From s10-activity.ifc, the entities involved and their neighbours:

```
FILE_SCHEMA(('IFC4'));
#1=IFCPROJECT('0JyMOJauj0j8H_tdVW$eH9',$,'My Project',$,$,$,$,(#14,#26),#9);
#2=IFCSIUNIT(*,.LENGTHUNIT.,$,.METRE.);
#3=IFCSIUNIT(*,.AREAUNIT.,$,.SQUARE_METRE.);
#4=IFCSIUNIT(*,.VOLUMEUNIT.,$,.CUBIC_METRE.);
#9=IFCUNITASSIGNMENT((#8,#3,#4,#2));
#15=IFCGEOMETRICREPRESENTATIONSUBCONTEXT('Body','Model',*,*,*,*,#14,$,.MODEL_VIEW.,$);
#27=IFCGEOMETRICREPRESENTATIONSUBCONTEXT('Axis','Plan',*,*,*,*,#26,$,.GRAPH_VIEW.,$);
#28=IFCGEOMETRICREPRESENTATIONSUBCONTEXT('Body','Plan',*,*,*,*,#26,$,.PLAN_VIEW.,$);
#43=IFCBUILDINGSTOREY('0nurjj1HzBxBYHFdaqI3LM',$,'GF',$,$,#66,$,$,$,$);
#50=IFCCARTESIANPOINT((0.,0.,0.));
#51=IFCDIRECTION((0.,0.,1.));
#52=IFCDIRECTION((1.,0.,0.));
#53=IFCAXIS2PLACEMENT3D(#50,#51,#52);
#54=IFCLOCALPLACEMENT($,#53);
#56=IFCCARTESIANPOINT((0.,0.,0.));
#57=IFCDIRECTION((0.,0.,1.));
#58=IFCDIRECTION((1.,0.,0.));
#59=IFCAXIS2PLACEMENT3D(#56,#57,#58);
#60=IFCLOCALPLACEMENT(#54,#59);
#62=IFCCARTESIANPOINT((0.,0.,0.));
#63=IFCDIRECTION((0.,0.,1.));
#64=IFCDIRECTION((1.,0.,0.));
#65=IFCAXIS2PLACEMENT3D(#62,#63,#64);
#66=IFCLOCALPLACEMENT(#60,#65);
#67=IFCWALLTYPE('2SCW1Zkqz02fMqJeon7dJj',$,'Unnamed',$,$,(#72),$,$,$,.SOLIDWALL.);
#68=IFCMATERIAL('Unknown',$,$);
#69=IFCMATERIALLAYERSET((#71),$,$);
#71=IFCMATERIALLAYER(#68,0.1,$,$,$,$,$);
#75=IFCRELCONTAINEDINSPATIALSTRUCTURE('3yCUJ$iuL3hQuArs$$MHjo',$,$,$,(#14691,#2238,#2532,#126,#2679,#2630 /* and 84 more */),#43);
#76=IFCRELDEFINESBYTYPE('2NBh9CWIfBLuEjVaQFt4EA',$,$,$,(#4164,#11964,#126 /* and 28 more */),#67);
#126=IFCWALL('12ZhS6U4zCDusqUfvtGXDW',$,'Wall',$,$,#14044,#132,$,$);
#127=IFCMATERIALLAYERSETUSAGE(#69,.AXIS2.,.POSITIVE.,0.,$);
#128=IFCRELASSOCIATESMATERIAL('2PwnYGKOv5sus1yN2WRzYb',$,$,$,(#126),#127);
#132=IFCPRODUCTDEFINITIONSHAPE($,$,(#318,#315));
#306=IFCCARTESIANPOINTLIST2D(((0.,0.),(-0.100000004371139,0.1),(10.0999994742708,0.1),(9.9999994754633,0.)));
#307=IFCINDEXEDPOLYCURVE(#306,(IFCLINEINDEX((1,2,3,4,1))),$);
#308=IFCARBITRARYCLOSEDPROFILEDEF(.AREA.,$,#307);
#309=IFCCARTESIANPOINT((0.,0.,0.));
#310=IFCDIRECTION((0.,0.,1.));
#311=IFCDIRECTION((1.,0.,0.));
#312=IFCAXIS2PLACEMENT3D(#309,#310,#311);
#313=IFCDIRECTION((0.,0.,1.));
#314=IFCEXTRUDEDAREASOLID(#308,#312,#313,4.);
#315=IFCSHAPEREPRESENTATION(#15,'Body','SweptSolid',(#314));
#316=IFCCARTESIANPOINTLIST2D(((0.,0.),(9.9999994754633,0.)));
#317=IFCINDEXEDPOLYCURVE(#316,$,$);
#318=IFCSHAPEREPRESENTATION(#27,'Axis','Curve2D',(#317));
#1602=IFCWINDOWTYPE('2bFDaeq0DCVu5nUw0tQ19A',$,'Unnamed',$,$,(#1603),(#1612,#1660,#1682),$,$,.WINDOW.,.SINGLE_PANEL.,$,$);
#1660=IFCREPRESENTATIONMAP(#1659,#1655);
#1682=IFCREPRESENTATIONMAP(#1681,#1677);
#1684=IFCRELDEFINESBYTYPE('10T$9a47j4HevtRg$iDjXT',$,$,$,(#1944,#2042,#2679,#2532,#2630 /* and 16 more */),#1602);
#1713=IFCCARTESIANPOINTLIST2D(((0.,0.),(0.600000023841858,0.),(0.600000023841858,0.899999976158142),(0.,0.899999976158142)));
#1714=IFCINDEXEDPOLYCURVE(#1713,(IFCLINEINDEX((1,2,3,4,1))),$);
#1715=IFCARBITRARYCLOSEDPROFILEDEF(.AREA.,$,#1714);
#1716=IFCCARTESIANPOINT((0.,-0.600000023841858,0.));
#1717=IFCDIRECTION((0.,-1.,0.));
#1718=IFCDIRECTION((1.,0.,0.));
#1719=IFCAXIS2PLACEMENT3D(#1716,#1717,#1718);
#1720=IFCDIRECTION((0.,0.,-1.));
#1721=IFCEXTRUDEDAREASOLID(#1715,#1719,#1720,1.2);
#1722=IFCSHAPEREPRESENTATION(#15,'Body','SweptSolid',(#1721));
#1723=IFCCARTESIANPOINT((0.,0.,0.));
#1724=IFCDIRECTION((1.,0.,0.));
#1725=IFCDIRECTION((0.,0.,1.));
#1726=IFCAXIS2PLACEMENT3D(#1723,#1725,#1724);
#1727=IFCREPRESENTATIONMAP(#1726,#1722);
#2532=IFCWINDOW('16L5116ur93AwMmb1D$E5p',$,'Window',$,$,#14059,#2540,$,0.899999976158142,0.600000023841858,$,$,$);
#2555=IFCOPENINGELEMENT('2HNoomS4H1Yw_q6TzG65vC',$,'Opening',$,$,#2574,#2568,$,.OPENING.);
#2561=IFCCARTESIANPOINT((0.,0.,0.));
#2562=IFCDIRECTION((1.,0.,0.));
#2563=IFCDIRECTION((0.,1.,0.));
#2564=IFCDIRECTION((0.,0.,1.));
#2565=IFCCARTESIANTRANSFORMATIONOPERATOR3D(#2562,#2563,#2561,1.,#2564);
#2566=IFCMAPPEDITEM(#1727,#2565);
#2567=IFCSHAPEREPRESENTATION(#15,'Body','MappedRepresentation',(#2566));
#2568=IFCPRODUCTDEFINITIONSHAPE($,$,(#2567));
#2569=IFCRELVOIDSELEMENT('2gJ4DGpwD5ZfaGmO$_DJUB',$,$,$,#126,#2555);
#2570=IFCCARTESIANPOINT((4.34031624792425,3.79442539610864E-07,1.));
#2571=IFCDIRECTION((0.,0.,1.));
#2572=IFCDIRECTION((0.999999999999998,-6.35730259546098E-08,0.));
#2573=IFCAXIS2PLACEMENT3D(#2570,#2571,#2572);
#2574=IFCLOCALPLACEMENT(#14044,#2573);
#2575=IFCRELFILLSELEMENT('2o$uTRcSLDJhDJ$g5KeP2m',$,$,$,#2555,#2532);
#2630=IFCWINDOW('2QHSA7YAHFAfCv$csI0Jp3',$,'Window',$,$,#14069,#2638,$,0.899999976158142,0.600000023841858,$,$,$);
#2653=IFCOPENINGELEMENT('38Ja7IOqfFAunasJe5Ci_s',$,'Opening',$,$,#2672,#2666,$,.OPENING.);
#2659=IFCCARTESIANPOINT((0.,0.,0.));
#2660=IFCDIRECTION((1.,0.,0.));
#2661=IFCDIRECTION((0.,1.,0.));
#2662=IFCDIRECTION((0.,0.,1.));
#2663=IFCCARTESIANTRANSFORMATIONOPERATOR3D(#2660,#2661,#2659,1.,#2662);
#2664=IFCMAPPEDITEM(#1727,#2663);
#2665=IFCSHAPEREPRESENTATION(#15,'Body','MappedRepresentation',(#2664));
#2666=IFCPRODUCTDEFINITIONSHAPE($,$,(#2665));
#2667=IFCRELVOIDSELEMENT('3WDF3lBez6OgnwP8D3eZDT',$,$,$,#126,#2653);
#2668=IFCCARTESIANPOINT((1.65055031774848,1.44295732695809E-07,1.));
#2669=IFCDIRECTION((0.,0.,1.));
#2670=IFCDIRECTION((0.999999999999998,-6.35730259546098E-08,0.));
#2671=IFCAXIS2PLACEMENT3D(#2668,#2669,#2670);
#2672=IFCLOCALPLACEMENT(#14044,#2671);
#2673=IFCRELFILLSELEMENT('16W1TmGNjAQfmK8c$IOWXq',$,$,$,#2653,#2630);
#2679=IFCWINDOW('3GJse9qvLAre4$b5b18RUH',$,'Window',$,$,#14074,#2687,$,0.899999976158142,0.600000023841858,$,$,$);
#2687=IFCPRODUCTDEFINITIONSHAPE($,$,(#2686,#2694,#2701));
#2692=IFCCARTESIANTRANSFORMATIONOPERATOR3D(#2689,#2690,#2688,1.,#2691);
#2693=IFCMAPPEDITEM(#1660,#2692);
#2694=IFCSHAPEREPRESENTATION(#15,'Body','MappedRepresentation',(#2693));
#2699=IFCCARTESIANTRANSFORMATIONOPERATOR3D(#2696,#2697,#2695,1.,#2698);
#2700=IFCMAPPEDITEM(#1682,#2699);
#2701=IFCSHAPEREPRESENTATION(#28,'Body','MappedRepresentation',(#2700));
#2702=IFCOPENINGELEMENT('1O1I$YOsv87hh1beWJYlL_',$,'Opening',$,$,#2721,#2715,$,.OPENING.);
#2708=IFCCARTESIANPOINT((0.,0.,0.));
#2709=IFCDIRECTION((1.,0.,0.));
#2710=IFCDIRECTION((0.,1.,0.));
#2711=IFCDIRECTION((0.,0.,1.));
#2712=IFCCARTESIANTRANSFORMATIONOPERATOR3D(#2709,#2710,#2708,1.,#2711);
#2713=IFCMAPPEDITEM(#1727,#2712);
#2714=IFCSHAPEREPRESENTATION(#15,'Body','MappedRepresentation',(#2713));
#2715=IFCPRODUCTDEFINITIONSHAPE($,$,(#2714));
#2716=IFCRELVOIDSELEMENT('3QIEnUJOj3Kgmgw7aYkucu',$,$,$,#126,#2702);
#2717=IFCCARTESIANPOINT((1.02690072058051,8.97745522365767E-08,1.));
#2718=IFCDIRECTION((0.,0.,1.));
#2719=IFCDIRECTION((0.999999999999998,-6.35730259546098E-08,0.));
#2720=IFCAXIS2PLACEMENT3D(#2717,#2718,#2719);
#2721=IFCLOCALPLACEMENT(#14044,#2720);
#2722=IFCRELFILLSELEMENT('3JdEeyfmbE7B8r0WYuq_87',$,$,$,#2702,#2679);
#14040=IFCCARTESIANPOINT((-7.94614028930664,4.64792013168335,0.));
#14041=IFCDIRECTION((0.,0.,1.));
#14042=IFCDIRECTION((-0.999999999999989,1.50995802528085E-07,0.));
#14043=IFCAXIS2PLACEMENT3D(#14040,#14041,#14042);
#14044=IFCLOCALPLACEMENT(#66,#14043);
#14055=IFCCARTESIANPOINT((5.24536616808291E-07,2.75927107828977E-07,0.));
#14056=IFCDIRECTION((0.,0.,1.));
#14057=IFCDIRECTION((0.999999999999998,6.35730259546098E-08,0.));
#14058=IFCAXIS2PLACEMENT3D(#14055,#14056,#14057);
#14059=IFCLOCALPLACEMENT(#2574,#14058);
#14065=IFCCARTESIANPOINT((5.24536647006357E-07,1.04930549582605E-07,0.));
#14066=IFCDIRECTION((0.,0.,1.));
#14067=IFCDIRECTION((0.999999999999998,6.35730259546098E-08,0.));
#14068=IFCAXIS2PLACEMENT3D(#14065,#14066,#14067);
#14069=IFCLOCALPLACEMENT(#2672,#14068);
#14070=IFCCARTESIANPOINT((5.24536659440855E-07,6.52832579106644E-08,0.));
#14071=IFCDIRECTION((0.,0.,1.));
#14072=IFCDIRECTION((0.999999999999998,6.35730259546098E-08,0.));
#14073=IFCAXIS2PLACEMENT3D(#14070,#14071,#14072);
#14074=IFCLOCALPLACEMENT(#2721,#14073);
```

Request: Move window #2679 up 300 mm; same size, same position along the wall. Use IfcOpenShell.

```python
import numpy as np
import ifcopenshell
import ifcopenshell.api.geometry
import ifcopenshell.util.placement
import ifcopenshell.util.unit

model = ifcopenshell.open("s10-activity.ifc")
unit_scale = ifcopenshell.util.unit.calculate_unit_scale(model)

window = model.by_id(2679)
opening = window.FillsVoids[0].RelatingOpeningElement
dz = 0.3

shift = np.array([0.0, 0.0, dz])
# The window is placed relative to its opening, so it follows when the opening moves.
matrix = ifcopenshell.util.placement.get_local_placement(opening.ObjectPlacement)
matrix[:3, 3] += shift
ifcopenshell.api.geometry.edit_object_placement(
    model, product=opening, matrix=matrix, is_si=False, should_transform_children=True
)

print(f"moved by {dz * unit_scale:+.3f} m")

model.write("s10-activity_rev.ifc")
```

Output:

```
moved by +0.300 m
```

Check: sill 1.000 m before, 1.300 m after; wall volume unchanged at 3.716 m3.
